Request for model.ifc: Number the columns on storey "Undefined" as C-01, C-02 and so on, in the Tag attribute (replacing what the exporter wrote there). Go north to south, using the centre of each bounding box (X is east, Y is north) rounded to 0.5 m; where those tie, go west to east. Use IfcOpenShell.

First a look at what the model holds.

```python
import ifcopenshell
import ifcopenshell.util.element
import ifcopenshell.util.placement

model = ifcopenshell.open("model.ifc")
print(model.schema)
storey = next(s for s in model.by_type("IfcBuildingStorey") if s.Name == "Undefined")
columns = [e for e in ifcopenshell.util.element.get_decomposition(storey) if e.is_a("IfcColumn")]
for e in sorted(columns, key=lambda e: e.id()):
    origin = ifcopenshell.util.placement.get_local_placement(e.ObjectPlacement)[:3, 3]
    print(e.id(), e.Tag, e.Name, origin.round(2) + 0.0, sep=" | ")
```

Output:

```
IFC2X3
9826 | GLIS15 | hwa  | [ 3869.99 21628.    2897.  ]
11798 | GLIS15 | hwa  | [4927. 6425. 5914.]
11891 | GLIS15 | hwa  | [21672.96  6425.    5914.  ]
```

```python
import ifcopenshell
import ifcopenshell.geom
import ifcopenshell.util.element
import ifcopenshell.util.shape

model = ifcopenshell.open("model.ifc")
settings = ifcopenshell.geom.settings()
settings.set("use-world-coords", True)


def centre(element):
    shape = ifcopenshell.geom.create_shape(settings, element)
    return ifcopenshell.util.shape.get_bbox_centroid(shape.geometry)


storey = next(s for s in model.by_type("IfcBuildingStorey") if s.Name == "Undefined")
columns = [e for e in ifcopenshell.util.element.get_decomposition(storey) if e.is_a("IfcColumn")]

# Insertion points can sit at a corner or the storey origin, so sort by the geometry (in metres).
centres = {e: centre(e) for e in columns}
columns.sort(key=lambda e: (-round(centres[e][1] / 0.5), centres[e][0]))

for i, e in enumerate(columns, start=1):
    number = f"C-{i:02d}"
    e.Tag = number
    print(e.id(), number)

model.write("model_edited.ifc")
```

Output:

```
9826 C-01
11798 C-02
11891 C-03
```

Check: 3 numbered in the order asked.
